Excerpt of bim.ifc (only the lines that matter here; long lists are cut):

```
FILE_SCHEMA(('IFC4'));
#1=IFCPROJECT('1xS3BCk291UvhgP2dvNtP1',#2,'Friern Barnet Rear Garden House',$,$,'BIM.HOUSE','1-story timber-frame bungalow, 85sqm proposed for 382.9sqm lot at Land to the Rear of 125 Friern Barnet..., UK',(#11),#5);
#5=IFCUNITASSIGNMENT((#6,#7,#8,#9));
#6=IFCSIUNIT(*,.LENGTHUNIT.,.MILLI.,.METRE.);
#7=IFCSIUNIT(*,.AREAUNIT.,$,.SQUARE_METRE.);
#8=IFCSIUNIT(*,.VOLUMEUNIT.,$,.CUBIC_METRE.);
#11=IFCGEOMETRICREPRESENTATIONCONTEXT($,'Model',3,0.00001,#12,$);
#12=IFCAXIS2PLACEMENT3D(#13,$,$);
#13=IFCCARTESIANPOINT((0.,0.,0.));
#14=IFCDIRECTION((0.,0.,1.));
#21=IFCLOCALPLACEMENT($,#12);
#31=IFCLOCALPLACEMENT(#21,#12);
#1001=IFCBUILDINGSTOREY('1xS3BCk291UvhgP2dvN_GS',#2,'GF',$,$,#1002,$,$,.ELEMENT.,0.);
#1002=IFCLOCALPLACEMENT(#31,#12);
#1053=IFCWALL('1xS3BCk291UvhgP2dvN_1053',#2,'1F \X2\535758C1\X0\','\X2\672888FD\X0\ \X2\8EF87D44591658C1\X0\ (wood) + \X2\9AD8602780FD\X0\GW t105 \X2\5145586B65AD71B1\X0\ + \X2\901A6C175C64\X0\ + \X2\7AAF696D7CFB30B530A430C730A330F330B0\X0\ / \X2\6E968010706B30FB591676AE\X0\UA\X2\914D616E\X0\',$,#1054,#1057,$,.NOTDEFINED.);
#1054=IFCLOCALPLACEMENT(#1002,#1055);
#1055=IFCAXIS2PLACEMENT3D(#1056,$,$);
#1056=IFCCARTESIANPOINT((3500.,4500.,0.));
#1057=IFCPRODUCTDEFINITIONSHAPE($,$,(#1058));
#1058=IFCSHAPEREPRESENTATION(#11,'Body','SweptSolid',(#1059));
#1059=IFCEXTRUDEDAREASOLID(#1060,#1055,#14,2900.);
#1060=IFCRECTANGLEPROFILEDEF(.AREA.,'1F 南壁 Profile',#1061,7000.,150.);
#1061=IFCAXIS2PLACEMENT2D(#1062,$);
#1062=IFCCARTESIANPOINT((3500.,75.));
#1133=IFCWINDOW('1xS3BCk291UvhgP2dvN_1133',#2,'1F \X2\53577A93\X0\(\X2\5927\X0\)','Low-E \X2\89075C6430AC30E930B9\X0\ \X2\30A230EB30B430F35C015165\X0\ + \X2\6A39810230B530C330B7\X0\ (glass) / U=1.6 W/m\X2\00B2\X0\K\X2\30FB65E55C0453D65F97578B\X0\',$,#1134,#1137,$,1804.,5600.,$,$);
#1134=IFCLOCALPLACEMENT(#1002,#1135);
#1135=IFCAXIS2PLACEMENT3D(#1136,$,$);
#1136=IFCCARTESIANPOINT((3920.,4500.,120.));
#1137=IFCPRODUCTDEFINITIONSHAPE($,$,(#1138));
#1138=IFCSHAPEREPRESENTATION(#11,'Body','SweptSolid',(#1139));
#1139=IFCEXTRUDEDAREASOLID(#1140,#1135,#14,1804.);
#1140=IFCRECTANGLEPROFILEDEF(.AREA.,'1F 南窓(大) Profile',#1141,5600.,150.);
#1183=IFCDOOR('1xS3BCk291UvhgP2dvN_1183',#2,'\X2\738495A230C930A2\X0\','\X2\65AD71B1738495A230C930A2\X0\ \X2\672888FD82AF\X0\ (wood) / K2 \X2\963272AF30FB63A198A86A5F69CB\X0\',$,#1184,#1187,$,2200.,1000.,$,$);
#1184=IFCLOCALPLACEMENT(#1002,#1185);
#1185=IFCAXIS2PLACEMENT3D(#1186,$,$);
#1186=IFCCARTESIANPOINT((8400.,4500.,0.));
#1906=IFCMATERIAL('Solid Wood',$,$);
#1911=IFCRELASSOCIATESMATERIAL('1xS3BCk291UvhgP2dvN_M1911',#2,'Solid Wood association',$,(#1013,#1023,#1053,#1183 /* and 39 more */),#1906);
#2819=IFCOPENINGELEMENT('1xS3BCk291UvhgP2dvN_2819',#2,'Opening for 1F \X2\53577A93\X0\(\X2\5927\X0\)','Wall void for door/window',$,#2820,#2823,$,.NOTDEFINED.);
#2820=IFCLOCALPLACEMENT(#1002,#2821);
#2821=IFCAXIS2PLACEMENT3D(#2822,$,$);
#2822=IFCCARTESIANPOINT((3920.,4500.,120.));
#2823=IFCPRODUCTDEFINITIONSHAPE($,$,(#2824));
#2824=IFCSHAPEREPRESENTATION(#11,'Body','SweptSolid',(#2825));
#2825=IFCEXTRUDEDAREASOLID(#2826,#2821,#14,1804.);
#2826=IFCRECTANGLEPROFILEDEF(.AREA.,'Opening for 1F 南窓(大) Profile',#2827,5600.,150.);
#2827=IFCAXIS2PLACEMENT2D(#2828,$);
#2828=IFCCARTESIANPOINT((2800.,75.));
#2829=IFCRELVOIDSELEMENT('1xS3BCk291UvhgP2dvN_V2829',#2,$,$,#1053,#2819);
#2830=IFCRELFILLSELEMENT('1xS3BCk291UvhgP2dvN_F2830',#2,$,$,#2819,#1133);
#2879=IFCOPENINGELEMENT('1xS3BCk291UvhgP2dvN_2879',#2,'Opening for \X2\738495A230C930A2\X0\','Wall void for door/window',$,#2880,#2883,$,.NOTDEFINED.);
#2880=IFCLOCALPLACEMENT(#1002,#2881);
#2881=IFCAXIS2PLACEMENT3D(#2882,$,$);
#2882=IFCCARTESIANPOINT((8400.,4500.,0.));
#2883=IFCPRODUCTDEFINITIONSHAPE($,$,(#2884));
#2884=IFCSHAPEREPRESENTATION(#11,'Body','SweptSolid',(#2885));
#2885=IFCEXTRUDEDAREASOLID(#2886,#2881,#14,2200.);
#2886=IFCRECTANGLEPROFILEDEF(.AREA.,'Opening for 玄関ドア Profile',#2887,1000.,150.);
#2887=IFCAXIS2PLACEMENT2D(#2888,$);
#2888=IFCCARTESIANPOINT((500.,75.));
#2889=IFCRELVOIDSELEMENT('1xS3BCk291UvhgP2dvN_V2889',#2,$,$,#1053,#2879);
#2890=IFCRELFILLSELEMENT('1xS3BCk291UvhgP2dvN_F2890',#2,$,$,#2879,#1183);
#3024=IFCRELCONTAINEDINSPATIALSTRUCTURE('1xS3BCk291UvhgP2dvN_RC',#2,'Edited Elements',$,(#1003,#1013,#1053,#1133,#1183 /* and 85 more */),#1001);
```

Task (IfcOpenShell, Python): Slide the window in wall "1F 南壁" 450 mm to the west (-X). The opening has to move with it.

```python
import ifcopenshell
import ifcopenshell.api.geometry
import ifcopenshell.util.placement
import ifcopenshell.util.unit

model = ifcopenshell.open("bim.ifc")
unit_scale = ifcopenshell.util.unit.calculate_unit_scale(model)

window = model.by_guid("1xS3BCk291UvhgP2dvN_1133")
opening = window.FillsVoids[0].RelatingOpeningElement
wall = opening.VoidsElements[0].RelatingBuildingElement

wall_matrix = ifcopenshell.util.placement.get_local_placement(wall.ObjectPlacement)
shift = wall_matrix[:3, 0] * -0.45 / unit_scale
before = ifcopenshell.util.placement.get_local_placement(window.ObjectPlacement)[:3, 3].copy()

# The window is not placed relative to its opening, so move both.
for product in (opening, window):
    matrix = ifcopenshell.util.placement.get_local_placement(product.ObjectPlacement)
    matrix[:3, 3] += shift
    ifcopenshell.api.geometry.edit_object_placement(model, product=product, matrix=matrix, is_si=False)

after = ifcopenshell.util.placement.get_local_placement(window.ObjectPlacement)[:3, 3]
print("window moved by", (after - before).round(3) + 0.0)

model.write("bim_rev.ifc")
```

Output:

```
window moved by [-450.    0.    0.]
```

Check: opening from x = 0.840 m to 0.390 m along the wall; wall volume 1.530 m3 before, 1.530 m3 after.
